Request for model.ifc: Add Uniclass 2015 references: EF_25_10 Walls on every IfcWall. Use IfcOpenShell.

First a look at what the model holds.

```python
import ifcopenshell

model = ifcopenshell.open("model.ifc")
print(model.schema)
print("classifications:", [c.Name for c in model.by_type("IfcClassification")])
for ifc_class in ("IfcDoor", "IfcRoof", "IfcStair", "IfcWall", "IfcWindow"):
    print(ifc_class, len(model.by_type(ifc_class)))
```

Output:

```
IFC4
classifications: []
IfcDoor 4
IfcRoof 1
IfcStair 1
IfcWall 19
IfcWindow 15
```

```python
import ifcopenshell
import ifcopenshell.api.classification

model = ifcopenshell.open("model.ifc")

system = ifcopenshell.api.classification.add_classification(model, classification="Uniclass 2015")

codes = {
    "IfcWall": ("EF_25_10", "Walls"),
}
for ifc_class, (code, name) in codes.items():
    products = model.by_type(ifc_class)
    ifcopenshell.api.classification.add_reference(
        model, products=products, classification=system, identification=code, name=name
    )
    print(code, len(products))

model.write("model_edited.ifc")
```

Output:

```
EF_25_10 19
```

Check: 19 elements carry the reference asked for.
